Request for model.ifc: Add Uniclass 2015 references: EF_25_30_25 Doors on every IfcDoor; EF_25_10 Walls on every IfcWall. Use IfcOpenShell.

First a look at what the model holds.

```python
import ifcopenshell

model = ifcopenshell.open("model.ifc")
print(model.schema)
print("classifications:", [c.Name for c in model.by_type("IfcClassification")])
for ifc_class in ("IfcDoor", "IfcRoof", "IfcStair", "IfcWall", "IfcWindow"):
    print(ifc_class, len(model.by_type(ifc_class)))
```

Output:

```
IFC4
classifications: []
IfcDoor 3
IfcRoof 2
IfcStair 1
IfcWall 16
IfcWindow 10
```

```python
import ifcopenshell
import ifcopenshell.api.classification

model = ifcopenshell.open("model.ifc")

system = ifcopenshell.api.classification.add_classification(model, classification="Uniclass 2015")

codes = {
    "IfcDoor": ("EF_25_30_25", "Doors"),
    "IfcWall": ("EF_25_10", "Walls"),
}
for ifc_class, (code, name) in codes.items():
    products = model.by_type(ifc_class)
    ifcopenshell.api.classification.add_reference(
        model, products=products, classification=system, identification=code, name=name
    )
    print(code, len(products))

model.write("model_v2.ifc")
```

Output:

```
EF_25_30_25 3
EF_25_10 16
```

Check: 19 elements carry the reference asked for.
